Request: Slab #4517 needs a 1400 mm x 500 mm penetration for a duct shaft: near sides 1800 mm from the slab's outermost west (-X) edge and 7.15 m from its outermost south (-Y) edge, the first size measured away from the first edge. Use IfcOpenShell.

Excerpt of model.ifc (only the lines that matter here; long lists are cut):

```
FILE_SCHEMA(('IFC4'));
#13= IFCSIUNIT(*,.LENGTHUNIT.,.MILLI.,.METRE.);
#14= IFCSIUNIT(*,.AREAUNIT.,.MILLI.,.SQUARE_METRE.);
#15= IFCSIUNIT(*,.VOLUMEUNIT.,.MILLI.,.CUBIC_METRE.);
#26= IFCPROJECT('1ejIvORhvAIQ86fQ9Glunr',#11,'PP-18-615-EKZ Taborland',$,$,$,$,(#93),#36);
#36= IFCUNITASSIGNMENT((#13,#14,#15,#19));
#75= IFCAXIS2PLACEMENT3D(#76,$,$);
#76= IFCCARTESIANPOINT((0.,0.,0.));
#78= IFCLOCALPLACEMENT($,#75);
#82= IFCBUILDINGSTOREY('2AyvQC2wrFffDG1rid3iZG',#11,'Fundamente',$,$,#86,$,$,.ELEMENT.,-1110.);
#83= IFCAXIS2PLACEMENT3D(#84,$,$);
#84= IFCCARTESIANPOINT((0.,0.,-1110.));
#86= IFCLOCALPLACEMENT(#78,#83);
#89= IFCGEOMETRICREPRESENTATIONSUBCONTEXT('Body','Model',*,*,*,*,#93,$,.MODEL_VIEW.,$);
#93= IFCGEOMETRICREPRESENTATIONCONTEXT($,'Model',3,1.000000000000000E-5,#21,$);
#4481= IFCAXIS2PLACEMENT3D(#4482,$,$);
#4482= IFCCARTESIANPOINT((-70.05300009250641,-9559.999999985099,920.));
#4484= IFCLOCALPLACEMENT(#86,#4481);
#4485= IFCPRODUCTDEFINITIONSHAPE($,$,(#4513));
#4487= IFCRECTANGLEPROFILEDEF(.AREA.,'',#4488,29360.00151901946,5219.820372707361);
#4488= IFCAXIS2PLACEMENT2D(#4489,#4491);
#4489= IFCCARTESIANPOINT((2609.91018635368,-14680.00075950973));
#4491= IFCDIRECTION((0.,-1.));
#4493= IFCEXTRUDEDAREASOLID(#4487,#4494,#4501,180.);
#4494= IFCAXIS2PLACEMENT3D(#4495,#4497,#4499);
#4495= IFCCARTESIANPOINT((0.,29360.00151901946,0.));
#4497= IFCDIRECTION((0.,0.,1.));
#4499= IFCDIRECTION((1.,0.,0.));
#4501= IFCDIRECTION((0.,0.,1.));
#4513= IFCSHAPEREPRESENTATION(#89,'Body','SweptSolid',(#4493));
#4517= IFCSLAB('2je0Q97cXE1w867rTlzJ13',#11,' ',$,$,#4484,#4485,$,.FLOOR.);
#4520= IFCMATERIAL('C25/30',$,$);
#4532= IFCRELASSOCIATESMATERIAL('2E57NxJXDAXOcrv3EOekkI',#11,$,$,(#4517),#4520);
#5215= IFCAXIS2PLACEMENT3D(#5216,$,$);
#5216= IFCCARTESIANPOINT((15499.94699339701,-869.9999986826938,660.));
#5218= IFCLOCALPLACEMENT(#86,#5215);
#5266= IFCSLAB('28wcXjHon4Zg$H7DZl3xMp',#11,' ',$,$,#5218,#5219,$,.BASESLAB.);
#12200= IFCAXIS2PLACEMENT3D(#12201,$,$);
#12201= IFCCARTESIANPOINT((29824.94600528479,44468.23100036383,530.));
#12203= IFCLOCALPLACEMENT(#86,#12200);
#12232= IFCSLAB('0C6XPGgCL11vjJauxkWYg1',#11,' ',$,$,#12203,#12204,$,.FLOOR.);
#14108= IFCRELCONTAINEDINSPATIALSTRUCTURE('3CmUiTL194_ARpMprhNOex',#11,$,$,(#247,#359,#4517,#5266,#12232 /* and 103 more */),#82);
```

```python
import numpy as np
import ifcopenshell
import ifcopenshell.api.feature
import ifcopenshell.api.geometry
import ifcopenshell.api.root
import ifcopenshell.geom
import ifcopenshell.util.placement
import ifcopenshell.util.representation
import ifcopenshell.util.shape
import ifcopenshell.util.unit

model = ifcopenshell.open("model.ifc")
unit_scale = ifcopenshell.util.unit.calculate_unit_scale(model)
settings = ifcopenshell.geom.settings()


def volume(element):
    """Net volume in cubic metres, openings subtracted."""
    shape = ifcopenshell.geom.create_shape(settings, element)
    return ifcopenshell.util.shape.get_volume(shape.geometry)


slab = model.by_id(4517)
before = volume(slab)

# Extent in the slab's own axes, in metres. The edges named are its -X and -Y sides.
slab_shape = ifcopenshell.geom.create_shape(settings, slab)
vertices = ifcopenshell.util.shape.get_vertices(slab_shape.geometry)
x_min, y_min, bottom = vertices.min(axis=0)
top = vertices[:, 2].max()

opening = ifcopenshell.api.root.create_entity(model, ifc_class="IfcOpeningElement", name="Duct shaft opening", predefined_type="OPENING")
context = ifcopenshell.util.representation.get_context(model, "Model", "Body", "MODEL_VIEW")
width, depth = 1.4, 0.5
outline = [(0.0, 0.0), (width, 0.0), (width, depth), (0.0, depth), (0.0, 0.0)]
# Overshoot both faces by 50 mm so the cut is clean.
shape = ifcopenshell.api.geometry.add_slab_representation(
    model, context=context, depth=top - bottom + 0.1, polyline=outline
)
ifcopenshell.api.geometry.assign_representation(model, product=opening, representation=shape)

matrix = ifcopenshell.util.placement.get_local_placement(slab.ObjectPlacement)
matrix[:, 3] = matrix @ np.append(np.array([x_min + 1.8, y_min + 7.15, bottom - 0.05]) / unit_scale, 1.0)
ifcopenshell.api.geometry.edit_object_placement(model, product=opening, matrix=matrix, is_si=False)
ifcopenshell.api.feature.add_feature(model, feature=opening, element=slab)

after = volume(slab)

print(f"slab volume {before:.3f} -> {after:.3f} m3")

model.write("model_v2.ifc")
```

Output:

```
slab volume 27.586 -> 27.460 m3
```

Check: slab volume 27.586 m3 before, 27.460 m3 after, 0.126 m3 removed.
